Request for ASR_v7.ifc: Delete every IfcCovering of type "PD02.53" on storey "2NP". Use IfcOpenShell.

First a look at what the model holds.

```python
import ifcopenshell
import ifcopenshell.util.element

model = ifcopenshell.open("ASR_v7.ifc")
print(model.schema)
storey = next(s for s in model.by_type("IfcBuildingStorey") if s.Name == "2NP")
coverings = [e for e in ifcopenshell.util.element.get_decomposition(storey) if e.is_a("IfcCovering")]
seen = {}
for e in coverings:
    element_type = ifcopenshell.util.element.get_type(e)
    name = element_type.Name if element_type not in (None, e) else None
    seen[name] = seen.get(name, 0) + 1
for name, count in sorted(seen.items(), key=str):
    print(count, "x", name)
```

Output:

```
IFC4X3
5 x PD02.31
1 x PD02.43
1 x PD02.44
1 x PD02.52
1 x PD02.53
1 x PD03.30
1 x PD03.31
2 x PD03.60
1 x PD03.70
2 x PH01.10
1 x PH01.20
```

```python
import ifcopenshell
import ifcopenshell.api.root
import ifcopenshell.util.element

model = ifcopenshell.open("ASR_v7.ifc")

storey = next(s for s in model.by_type("IfcBuildingStorey") if s.Name == "2NP")
coverings = [e for e in ifcopenshell.util.element.get_decomposition(storey) if e.is_a("IfcCovering")]
targets = [e for e in coverings if (t := ifcopenshell.util.element.get_type(e)) not in (None, e) and t.Name == "PD02.53"]

for e in targets:
    ifcopenshell.api.root.remove_product(model, product=e)
print(len(targets), "removed")

model.write("ASR_v7_v2.ifc")
```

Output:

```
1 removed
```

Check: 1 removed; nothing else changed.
